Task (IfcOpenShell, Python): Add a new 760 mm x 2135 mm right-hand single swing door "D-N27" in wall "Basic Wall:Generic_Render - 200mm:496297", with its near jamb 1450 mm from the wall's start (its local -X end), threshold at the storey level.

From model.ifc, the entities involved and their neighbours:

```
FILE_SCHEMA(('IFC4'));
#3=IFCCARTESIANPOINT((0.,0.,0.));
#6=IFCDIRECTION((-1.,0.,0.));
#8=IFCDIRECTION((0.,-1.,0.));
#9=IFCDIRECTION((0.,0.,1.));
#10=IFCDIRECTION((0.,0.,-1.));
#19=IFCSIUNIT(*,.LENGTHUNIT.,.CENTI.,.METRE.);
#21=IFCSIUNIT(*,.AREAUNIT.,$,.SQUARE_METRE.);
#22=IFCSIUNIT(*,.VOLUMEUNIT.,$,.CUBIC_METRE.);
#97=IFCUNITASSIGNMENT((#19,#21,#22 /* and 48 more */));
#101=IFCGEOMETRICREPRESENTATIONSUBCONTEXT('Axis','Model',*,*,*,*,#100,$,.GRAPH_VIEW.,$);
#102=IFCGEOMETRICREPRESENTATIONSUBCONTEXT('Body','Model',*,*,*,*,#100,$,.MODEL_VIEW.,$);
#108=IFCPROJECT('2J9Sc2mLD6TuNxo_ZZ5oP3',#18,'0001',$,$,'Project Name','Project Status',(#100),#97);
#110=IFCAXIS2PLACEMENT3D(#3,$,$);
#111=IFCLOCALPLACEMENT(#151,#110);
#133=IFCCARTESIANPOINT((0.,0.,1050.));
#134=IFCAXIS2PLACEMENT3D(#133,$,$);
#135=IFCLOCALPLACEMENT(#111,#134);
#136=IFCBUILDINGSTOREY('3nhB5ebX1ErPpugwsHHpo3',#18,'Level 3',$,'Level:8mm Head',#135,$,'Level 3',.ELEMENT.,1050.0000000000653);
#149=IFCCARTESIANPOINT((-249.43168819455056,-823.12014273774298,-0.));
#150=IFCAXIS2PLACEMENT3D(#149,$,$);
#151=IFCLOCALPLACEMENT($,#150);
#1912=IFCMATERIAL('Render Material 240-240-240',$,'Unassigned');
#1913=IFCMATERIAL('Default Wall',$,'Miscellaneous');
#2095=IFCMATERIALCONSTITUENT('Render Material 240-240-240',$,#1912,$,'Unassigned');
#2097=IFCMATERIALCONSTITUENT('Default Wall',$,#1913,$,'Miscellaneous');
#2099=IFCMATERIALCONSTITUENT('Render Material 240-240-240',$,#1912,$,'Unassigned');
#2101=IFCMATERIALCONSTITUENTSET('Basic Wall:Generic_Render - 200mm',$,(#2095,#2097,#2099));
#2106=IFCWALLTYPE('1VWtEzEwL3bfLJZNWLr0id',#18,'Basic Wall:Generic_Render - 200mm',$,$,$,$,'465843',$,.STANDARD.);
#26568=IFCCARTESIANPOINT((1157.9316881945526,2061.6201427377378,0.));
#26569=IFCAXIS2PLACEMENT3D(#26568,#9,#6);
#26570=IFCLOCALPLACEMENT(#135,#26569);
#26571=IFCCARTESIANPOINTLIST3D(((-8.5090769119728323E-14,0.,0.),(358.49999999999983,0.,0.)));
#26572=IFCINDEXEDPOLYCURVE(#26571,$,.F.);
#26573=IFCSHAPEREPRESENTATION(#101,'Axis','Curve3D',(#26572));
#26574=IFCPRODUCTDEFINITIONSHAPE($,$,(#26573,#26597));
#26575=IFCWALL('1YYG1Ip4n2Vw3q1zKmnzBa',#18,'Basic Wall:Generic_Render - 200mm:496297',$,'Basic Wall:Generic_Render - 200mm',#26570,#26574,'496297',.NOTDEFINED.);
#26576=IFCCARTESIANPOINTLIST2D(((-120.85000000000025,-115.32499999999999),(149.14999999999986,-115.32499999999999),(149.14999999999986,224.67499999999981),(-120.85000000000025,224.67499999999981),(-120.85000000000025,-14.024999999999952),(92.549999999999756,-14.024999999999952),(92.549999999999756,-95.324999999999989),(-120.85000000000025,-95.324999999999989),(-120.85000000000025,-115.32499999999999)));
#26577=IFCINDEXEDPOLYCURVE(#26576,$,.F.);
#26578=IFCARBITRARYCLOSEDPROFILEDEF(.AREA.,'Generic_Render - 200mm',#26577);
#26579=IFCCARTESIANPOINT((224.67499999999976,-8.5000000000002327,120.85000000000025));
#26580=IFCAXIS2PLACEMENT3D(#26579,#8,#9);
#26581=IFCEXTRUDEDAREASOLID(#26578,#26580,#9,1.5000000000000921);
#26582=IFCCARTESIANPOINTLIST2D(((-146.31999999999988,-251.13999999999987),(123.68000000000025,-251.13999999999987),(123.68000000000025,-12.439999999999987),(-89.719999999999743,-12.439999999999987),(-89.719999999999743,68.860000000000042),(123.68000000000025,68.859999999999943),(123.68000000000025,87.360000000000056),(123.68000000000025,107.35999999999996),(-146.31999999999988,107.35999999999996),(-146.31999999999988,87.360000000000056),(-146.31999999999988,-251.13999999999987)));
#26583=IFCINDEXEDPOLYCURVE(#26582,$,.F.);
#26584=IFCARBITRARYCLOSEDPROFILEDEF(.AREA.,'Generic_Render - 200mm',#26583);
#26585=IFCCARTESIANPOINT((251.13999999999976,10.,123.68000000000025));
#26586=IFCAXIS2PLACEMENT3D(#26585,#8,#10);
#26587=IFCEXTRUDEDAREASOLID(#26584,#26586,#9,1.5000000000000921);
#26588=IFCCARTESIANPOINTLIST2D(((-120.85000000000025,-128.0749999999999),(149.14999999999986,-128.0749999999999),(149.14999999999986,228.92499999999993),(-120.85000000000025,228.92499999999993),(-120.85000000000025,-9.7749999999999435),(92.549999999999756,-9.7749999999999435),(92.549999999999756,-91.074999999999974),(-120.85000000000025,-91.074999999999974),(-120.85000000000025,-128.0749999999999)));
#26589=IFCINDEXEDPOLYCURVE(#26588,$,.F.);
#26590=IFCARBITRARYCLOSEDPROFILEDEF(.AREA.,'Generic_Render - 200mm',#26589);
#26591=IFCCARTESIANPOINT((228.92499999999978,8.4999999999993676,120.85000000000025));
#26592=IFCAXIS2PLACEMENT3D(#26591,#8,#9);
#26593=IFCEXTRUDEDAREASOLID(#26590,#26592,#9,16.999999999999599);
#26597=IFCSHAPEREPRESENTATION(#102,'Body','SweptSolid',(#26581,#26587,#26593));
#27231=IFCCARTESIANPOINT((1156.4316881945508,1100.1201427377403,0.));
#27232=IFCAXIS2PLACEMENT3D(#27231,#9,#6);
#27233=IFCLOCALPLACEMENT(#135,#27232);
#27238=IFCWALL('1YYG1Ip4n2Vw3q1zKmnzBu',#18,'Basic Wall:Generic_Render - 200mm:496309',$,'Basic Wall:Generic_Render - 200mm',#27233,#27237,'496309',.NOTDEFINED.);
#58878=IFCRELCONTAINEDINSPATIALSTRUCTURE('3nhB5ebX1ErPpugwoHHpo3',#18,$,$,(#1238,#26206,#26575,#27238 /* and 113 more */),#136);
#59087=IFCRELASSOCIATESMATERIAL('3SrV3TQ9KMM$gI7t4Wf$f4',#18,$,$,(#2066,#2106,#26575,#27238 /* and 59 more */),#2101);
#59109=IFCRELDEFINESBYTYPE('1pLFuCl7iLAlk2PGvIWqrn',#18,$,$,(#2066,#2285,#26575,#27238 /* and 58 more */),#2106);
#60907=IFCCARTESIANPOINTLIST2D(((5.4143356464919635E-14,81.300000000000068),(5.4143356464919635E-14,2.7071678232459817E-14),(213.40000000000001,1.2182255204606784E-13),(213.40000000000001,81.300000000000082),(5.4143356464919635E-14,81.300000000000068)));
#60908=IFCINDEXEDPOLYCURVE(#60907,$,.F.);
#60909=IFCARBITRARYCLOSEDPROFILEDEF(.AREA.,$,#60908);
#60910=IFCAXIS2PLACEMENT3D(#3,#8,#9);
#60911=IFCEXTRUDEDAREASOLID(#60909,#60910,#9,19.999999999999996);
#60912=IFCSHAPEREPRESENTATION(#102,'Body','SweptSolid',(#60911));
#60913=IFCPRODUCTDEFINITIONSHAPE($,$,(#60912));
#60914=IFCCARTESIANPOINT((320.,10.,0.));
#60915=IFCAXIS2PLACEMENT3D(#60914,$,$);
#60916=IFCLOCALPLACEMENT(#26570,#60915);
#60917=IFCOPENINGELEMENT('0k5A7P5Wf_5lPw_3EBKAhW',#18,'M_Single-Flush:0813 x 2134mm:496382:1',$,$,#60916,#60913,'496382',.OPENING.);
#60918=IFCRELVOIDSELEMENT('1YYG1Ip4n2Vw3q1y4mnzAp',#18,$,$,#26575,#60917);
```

```python
import numpy as np
import ifcopenshell
import ifcopenshell.api.feature
import ifcopenshell.api.geometry
import ifcopenshell.api.root
import ifcopenshell.api.spatial
import ifcopenshell.geom
import ifcopenshell.util.element
import ifcopenshell.util.placement
import ifcopenshell.util.representation
import ifcopenshell.util.shape
import ifcopenshell.util.unit

model = ifcopenshell.open("model.ifc")
unit_scale = ifcopenshell.util.unit.calculate_unit_scale(model)
settings = ifcopenshell.geom.settings()


def volume(element):
    """Net volume in cubic metres, openings subtracted."""
    shape = ifcopenshell.geom.create_shape(settings, element)
    return ifcopenshell.util.shape.get_volume(shape.geometry)


wall = model.by_guid("1YYG1Ip4n2Vw3q1zKmnzBa")
storey = ifcopenshell.util.element.get_container(wall, ifc_class="IfcBuildingStorey")
context = ifcopenshell.util.representation.get_context(model, "Model", "Body", "MODEL_VIEW")
before = volume(wall)

width, height, from_end, sill = 0.76, 2.135, 1.45, 0.0  # metres

# The wall runs along its own X axis, and the end named is its -X end.
wall_shape = ifcopenshell.geom.create_shape(settings, wall)
x, y, z = ifcopenshell.util.shape.get_vertices(wall_shape.geometry).T
start = x.min() + from_end
face, thickness = float(y.min()), float(y.max() - y.min())
wall_matrix = ifcopenshell.util.placement.get_local_placement(wall.ObjectPlacement)
level = ifcopenshell.util.placement.get_local_placement(storey.ObjectPlacement)[2, 3]


def in_wall(x, y):
    """Placement at x, y metres in the wall's axes, at sill height."""
    matrix = wall_matrix.copy()
    matrix[:, 3] = wall_matrix @ np.array([x / unit_scale, y / unit_scale, 0.0, 1.0])
    matrix[2, 3] = level + sill / unit_scale
    return matrix


# Opening: a box that overshoots both wall faces by 50 mm.
opening = ifcopenshell.api.root.create_entity(model, ifc_class="IfcOpeningElement", predefined_type="OPENING")
box = ifcopenshell.api.geometry.add_wall_representation(
    model, context=context, length=width, height=height, thickness=thickness + 0.1
)
ifcopenshell.api.geometry.assign_representation(model, product=opening, representation=box)
ifcopenshell.api.geometry.edit_object_placement(model, product=opening, matrix=in_wall(start, face - 0.05), is_si=False)
ifcopenshell.api.feature.add_feature(model, feature=opening, element=wall)

door = ifcopenshell.api.root.create_entity(model, ifc_class="IfcDoor", name="D-N27", predefined_type="DOOR")
door.OverallWidth, door.OverallHeight = width / unit_scale, height / unit_scale
door.OperationType = "SINGLE_SWING_RIGHT"
body = ifcopenshell.api.geometry.add_door_representation(
    model,
    context=context,
    overall_width=door.OverallWidth,
    overall_height=door.OverallHeight,
    operation_type="SINGLE_SWING_RIGHT",
    lining_properties={"LiningDepth": thickness / unit_scale, "ThresholdDepth": thickness / unit_scale},
)
ifcopenshell.api.geometry.assign_representation(model, product=door, representation=body)
ifcopenshell.api.spatial.assign_container(model, products=[door], relating_structure=storey)
ifcopenshell.api.feature.add_filling(model, opening=opening, element=door)

# The lining spans the wall, so the door starts at the wall face.
ifcopenshell.api.geometry.edit_object_placement(model, product=door, matrix=in_wall(start, face), is_si=False)

after = volume(wall)

print(f"wall volume {before:.3f} -> {after:.3f} m3")

model.write("model-out.ifc")
```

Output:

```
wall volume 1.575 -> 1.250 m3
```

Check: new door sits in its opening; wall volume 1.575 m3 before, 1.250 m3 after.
